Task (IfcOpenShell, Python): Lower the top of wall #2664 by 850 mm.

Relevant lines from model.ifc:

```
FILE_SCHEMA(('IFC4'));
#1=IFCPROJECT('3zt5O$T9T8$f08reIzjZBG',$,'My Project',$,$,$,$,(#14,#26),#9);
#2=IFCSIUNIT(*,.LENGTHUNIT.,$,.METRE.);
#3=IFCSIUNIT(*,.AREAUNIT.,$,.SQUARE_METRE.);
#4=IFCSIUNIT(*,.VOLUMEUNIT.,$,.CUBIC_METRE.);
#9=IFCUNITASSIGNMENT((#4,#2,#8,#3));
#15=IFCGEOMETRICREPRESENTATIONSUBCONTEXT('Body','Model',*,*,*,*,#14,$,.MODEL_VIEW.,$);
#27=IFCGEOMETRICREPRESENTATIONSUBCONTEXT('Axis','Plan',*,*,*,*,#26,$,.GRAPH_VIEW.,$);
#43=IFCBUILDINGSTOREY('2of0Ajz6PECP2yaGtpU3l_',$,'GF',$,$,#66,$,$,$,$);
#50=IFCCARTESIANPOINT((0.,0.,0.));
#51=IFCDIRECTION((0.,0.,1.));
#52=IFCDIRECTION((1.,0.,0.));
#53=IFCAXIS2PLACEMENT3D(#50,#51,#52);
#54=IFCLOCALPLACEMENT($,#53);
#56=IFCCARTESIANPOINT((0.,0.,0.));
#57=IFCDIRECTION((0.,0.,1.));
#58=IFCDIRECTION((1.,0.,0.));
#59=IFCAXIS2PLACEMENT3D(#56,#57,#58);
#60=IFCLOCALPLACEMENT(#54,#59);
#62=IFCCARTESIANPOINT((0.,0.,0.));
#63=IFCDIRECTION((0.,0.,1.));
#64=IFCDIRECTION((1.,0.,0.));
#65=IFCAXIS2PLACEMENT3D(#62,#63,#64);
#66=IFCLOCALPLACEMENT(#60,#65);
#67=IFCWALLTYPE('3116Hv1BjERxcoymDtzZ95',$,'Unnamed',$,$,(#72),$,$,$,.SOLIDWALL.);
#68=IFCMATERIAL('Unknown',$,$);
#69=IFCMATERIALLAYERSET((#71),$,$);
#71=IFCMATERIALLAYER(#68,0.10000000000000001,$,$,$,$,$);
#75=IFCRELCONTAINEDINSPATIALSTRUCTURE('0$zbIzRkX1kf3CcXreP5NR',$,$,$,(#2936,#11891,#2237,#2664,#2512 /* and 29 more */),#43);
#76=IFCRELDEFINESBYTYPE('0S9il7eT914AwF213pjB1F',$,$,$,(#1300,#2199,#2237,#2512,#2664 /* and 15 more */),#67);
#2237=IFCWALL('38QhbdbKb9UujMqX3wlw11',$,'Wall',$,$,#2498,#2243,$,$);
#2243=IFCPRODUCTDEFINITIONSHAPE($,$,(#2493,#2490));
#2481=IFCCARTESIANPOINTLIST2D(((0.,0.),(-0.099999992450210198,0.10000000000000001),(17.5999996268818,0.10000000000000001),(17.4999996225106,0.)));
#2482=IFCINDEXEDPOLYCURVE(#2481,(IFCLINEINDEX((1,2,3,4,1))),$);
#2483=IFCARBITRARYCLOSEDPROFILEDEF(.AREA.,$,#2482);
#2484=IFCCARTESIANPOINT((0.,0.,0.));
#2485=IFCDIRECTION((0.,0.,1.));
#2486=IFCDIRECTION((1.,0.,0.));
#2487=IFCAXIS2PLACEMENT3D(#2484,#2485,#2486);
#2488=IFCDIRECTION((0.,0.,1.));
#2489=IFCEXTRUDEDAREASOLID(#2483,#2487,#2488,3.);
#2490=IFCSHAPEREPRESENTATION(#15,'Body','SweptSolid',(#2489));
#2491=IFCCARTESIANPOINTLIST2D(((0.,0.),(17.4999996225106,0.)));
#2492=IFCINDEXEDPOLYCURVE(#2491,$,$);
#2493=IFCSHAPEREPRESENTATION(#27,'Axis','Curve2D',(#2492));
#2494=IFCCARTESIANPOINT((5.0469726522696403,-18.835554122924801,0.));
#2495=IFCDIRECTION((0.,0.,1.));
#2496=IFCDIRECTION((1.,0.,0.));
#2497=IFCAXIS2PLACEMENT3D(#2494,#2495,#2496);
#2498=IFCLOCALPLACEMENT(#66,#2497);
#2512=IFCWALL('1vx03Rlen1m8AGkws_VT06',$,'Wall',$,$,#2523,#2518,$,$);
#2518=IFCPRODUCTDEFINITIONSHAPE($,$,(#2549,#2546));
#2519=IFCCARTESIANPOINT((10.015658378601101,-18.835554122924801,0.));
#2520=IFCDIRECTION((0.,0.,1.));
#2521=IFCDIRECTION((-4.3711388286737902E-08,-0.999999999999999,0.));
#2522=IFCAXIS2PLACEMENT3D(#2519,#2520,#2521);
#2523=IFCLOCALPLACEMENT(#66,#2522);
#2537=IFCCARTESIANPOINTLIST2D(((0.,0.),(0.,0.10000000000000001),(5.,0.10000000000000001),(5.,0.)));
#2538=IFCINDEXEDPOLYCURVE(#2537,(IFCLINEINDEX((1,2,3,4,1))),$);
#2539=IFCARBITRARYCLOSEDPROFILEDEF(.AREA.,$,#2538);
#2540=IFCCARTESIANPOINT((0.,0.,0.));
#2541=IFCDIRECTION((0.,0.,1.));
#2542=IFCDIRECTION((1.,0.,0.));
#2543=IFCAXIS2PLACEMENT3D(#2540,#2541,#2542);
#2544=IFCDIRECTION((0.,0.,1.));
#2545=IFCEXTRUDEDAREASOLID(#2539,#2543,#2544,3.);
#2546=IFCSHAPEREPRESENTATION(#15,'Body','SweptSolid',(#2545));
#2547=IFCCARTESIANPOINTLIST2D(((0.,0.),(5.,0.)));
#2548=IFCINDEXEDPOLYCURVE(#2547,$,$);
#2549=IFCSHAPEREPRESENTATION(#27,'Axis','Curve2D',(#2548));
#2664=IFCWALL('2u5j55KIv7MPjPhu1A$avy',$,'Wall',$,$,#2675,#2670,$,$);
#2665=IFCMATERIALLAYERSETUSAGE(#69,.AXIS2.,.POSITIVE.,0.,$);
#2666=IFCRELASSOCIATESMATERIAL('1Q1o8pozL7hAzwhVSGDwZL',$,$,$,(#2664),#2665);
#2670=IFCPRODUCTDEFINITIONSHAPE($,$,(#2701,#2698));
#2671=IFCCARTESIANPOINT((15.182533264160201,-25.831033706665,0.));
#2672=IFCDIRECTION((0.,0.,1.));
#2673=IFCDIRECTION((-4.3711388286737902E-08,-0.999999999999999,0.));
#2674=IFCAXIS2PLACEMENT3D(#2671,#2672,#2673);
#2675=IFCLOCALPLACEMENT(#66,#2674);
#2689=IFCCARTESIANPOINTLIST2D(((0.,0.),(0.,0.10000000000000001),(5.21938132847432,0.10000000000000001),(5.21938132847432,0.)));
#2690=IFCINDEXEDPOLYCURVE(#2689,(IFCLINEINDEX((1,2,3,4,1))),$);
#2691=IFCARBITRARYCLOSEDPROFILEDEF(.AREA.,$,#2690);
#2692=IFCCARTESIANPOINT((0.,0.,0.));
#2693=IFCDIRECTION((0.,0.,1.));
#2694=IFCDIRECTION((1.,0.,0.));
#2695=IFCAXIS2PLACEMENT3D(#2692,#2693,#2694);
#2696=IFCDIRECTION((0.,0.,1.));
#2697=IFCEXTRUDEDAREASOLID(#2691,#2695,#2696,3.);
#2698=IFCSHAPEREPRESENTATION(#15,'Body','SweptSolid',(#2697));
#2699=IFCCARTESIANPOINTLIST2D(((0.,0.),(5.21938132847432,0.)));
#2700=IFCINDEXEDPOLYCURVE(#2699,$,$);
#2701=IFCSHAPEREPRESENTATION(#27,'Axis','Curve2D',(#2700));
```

```python
import ifcopenshell
import ifcopenshell.geom
import ifcopenshell.util.representation
import ifcopenshell.util.shape

model = ifcopenshell.open("model.ifc")
settings = ifcopenshell.geom.settings()


def volume(element):
    """Net volume in cubic metres, openings subtracted."""
    shape = ifcopenshell.geom.create_shape(settings, element)
    return ifcopenshell.util.shape.get_volume(shape.geometry)


wall = model.by_guid("2u5j55KIv7MPjPhu1A$avy")
before = volume(wall)

body = ifcopenshell.util.representation.get_representation(wall, "Model", "Body")
solid = body.Items[0]
old_height = solid.Depth
solid.Depth -= 0.85
after = volume(wall)

print(f"height {old_height:g} -> {solid.Depth:g}, volume {before:.3f} -> {after:.3f} m3")

model.write("model_edited.ifc")
```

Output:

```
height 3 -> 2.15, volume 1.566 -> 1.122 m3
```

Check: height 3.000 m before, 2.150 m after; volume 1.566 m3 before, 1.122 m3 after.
